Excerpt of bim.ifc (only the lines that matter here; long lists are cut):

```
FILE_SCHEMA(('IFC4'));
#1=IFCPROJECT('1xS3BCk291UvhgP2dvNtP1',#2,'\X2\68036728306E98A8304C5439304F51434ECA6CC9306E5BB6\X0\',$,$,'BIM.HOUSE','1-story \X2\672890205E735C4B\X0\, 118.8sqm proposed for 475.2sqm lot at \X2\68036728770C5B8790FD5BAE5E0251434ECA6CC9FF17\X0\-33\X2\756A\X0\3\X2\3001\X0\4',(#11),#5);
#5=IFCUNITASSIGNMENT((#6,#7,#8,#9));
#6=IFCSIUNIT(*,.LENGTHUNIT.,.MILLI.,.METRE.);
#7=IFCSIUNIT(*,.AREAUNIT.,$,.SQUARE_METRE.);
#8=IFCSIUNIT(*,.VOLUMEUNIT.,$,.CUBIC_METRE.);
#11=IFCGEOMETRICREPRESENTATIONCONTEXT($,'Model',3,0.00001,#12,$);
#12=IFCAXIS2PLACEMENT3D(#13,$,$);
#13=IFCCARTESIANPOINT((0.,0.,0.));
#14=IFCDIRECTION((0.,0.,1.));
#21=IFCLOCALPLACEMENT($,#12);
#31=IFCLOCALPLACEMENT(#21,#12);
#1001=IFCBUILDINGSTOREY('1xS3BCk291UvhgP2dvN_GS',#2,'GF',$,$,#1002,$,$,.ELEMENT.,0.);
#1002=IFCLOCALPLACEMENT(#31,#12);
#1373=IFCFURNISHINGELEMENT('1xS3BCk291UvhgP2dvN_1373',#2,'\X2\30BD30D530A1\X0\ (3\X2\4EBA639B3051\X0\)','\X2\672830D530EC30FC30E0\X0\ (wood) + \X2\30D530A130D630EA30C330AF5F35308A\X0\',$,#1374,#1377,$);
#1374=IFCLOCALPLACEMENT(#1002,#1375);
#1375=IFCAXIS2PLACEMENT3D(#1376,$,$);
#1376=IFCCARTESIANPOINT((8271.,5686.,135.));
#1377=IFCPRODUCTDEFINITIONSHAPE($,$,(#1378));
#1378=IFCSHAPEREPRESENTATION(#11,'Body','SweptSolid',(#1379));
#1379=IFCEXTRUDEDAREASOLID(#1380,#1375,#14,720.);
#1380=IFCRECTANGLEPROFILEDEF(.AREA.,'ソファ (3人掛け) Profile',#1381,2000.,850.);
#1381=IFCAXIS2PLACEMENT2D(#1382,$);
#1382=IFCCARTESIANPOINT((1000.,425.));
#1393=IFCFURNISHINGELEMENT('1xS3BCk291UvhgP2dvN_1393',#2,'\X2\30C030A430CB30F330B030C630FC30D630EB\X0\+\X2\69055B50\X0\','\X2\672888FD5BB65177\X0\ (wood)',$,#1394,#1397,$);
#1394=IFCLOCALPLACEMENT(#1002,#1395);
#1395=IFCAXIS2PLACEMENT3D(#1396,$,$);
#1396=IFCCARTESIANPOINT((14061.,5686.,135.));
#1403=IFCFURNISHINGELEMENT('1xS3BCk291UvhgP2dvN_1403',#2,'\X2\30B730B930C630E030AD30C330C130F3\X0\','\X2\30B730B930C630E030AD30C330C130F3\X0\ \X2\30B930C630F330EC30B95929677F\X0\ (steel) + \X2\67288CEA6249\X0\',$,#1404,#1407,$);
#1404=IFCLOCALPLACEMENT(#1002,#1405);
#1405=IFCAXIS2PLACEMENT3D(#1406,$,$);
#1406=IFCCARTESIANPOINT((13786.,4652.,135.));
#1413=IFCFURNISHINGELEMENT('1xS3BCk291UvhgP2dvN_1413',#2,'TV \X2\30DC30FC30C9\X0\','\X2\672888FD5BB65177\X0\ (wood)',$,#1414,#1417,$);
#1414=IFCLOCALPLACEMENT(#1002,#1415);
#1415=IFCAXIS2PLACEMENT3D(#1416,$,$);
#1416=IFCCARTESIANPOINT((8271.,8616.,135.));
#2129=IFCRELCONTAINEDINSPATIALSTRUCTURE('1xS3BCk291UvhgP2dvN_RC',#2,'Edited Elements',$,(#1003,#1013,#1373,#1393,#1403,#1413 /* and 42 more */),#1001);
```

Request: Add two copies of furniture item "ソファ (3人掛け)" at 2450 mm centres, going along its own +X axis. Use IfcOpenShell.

```python
import ifcopenshell
import ifcopenshell.api.geometry
import ifcopenshell.api.root
import ifcopenshell.util.element
import ifcopenshell.util.placement
import ifcopenshell.util.unit

model = ifcopenshell.open("bim.ifc")
unit_scale = ifcopenshell.util.unit.calculate_unit_scale(model)


def reuse_history(source, copy):
    """copy_class also copies each property set's owner history, people and application; keep the originals."""
    for rel in copy.IsDefinedBy:
        if rel.is_a("IfcRelDefinesByProperties") and (history := rel.RelatingPropertyDefinition.OwnerHistory):
            rel.RelatingPropertyDefinition.OwnerHistory = source.OwnerHistory
            ifcopenshell.util.element.remove_deep2(model, history)


source = model.by_id(1373)
base = ifcopenshell.util.placement.get_local_placement(source.ObjectPlacement)
step = base[:3, 0] * 2.45 / unit_scale

for i in range(1, 3):
    copy = ifcopenshell.api.root.copy_class(model, product=source)
    copy.Representation = ifcopenshell.util.element.copy_deep(
        model, source.Representation, exclude=["IfcGeometricRepresentationContext", "IfcRepresentationMap"]
    )
    reuse_history(source, copy)
    matrix = base.copy()
    matrix[:3, 3] += i * step
    print("added at", matrix[:3, 3].round(3) + 0.0)
    ifcopenshell.api.geometry.edit_object_placement(model, product=copy, matrix=matrix, is_si=False)

model.write("bim_edited.ifc")
```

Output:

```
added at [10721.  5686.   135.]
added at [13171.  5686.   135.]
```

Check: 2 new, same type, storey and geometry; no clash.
